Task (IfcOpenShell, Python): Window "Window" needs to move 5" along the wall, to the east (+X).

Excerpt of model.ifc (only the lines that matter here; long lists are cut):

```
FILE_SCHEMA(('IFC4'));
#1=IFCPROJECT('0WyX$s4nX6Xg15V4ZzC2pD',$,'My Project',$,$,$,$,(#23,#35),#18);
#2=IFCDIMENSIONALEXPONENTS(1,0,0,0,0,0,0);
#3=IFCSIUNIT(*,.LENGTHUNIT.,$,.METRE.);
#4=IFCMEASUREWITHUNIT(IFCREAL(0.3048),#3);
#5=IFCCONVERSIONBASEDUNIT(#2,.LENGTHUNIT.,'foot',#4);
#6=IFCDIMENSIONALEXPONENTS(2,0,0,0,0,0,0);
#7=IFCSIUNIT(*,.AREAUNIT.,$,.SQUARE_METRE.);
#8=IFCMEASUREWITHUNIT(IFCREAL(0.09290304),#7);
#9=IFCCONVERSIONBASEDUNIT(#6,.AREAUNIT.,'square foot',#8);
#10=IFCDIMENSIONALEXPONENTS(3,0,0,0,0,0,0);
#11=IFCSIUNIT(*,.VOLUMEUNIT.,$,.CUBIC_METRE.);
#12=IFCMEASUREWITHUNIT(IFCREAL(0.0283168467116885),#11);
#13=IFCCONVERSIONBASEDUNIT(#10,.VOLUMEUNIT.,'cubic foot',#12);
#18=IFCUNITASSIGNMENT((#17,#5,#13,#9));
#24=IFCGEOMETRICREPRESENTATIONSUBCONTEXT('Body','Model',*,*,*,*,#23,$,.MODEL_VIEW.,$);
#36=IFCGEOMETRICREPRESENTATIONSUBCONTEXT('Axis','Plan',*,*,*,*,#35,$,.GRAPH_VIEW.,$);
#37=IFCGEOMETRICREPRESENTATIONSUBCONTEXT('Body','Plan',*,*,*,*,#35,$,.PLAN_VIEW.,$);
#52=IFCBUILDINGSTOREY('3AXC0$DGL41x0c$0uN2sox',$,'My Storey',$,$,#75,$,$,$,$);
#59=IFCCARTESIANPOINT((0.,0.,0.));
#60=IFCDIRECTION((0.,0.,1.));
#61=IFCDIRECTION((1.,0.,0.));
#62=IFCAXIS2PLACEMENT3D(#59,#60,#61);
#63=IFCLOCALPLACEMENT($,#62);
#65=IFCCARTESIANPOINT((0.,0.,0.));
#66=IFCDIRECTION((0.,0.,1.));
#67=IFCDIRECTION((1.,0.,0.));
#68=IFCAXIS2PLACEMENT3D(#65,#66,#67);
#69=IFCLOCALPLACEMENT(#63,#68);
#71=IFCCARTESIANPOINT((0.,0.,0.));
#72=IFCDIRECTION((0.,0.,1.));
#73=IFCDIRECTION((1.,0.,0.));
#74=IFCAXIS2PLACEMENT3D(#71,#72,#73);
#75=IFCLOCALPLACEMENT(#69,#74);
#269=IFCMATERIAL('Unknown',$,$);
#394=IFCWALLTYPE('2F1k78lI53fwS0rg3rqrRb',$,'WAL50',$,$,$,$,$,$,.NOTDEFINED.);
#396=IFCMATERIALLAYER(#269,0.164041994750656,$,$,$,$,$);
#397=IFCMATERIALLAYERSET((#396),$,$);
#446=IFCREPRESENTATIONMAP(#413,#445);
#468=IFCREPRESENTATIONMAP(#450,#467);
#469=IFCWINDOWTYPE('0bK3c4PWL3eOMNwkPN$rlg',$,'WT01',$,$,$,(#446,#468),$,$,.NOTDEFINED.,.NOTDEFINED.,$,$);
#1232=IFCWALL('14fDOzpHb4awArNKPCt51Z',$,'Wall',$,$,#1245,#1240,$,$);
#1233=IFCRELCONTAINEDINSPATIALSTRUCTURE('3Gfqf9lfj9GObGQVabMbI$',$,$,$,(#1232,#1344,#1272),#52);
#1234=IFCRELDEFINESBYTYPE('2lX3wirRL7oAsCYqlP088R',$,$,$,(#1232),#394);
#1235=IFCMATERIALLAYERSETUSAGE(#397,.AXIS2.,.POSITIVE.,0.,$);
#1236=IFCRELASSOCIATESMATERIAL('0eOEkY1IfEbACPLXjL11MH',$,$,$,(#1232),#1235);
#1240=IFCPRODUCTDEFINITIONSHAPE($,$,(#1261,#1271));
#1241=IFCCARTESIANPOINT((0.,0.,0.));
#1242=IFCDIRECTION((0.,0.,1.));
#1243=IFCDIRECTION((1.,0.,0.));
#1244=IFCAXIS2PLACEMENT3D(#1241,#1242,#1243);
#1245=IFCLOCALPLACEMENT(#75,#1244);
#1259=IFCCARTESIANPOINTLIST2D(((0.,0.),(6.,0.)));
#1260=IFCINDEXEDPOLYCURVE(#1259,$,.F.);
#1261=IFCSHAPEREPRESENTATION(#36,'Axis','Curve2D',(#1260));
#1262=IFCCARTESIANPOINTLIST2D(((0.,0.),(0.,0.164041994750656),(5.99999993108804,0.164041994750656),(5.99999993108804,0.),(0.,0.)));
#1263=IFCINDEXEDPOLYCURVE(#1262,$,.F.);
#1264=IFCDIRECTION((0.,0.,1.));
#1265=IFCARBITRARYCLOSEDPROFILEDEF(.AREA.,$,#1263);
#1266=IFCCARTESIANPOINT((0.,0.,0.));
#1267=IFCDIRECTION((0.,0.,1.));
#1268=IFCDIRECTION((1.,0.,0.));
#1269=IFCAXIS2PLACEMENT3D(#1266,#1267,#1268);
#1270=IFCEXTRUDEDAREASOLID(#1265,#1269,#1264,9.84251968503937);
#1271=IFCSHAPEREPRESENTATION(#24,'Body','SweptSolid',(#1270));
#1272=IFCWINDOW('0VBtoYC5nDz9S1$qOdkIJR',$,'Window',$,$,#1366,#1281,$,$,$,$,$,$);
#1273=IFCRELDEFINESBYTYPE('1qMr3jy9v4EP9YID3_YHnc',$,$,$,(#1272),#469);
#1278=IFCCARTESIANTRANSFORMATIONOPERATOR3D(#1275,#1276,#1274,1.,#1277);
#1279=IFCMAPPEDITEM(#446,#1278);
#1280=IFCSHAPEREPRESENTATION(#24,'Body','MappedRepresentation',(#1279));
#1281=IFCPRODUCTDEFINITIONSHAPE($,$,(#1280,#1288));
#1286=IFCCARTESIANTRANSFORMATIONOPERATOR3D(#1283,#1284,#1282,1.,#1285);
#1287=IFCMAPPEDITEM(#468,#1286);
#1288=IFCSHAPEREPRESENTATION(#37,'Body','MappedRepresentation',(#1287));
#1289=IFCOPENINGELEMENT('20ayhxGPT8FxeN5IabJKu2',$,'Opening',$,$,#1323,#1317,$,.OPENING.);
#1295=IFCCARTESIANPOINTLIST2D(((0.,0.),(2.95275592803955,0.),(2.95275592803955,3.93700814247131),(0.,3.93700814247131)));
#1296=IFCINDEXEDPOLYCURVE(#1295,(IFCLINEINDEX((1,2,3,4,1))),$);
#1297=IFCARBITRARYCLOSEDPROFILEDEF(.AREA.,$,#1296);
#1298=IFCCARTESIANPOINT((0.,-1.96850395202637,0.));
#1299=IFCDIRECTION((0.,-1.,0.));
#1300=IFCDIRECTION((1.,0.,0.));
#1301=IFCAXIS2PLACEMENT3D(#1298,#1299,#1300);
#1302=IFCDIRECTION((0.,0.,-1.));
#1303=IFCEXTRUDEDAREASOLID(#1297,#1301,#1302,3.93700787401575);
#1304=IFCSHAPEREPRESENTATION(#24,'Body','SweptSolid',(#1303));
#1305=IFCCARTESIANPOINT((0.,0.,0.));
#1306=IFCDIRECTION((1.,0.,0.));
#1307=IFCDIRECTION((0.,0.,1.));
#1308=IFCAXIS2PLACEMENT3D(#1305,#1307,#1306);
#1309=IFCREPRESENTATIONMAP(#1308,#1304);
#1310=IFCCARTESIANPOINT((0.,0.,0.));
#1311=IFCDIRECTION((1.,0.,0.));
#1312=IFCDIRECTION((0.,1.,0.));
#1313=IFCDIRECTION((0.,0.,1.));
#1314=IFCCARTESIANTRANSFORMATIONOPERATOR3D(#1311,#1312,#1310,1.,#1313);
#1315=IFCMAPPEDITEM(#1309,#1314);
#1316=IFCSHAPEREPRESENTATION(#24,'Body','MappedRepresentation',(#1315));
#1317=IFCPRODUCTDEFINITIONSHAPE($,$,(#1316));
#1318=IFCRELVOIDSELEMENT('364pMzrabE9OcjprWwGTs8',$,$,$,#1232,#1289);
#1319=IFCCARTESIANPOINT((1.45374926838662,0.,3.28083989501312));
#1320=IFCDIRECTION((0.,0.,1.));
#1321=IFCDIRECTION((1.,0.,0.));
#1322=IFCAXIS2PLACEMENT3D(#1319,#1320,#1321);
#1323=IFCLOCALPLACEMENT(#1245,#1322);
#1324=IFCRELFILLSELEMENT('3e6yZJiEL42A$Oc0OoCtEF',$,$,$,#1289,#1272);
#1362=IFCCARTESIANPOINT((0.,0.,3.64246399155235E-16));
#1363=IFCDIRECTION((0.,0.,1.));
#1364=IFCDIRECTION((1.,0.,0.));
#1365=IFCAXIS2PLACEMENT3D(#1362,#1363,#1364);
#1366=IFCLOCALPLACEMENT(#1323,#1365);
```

```python
import ifcopenshell
import ifcopenshell.api.geometry
import ifcopenshell.util.placement
import ifcopenshell.util.unit

model = ifcopenshell.open("model.ifc")
unit_scale = ifcopenshell.util.unit.calculate_unit_scale(model)

window = model.by_guid("0VBtoYC5nDz9S1$qOdkIJR")
opening = window.FillsVoids[0].RelatingOpeningElement
wall = opening.VoidsElements[0].RelatingBuildingElement

wall_matrix = ifcopenshell.util.placement.get_local_placement(wall.ObjectPlacement)
shift = wall_matrix[:3, 0] * 5 * 0.0254 / unit_scale
before = ifcopenshell.util.placement.get_local_placement(window.ObjectPlacement)[:3, 3].copy()

# The window is placed relative to its opening, so it follows when the opening moves.
matrix = ifcopenshell.util.placement.get_local_placement(opening.ObjectPlacement)
matrix[:3, 3] += shift
ifcopenshell.api.geometry.edit_object_placement(
    model, product=opening, matrix=matrix, is_si=False, should_transform_children=True
)

after = ifcopenshell.util.placement.get_local_placement(window.ObjectPlacement)[:3, 3]
print("window moved by", (after - before).round(3) + 0.0)

model.write("model_edited.ifc")
```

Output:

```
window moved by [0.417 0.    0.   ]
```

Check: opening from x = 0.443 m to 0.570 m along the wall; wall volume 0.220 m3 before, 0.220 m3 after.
